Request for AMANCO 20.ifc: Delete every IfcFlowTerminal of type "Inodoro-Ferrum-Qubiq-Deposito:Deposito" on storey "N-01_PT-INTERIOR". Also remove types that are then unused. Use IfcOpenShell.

First a look at what the model holds.

```python
import ifcopenshell
import ifcopenshell.util.element

model = ifcopenshell.open("AMANCO 20.ifc")
print(model.schema)
storey = next(s for s in model.by_type("IfcBuildingStorey") if s.Name == "N-01_PT-INTERIOR")
terminals = [e for e in ifcopenshell.util.element.get_decomposition(storey) if e.is_a("IfcFlowTerminal")]
seen = {}
for e in terminals:
    element_type = ifcopenshell.util.element.get_type(e)
    name = element_type.Name if element_type not in (None, e) else None
    seen[name] = seen.get(name, 0) + 1
for name, count in sorted(seen.items(), key=str):
    print(count, "x", name)
```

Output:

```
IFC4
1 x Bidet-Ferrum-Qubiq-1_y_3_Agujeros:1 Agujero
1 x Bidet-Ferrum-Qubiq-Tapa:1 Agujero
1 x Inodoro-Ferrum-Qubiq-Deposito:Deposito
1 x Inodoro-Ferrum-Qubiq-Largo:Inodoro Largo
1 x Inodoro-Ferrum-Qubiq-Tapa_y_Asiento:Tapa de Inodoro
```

```python
import ifcopenshell
import ifcopenshell.api.root
import ifcopenshell.util.element

model = ifcopenshell.open("AMANCO 20.ifc")

storey = next(s for s in model.by_type("IfcBuildingStorey") if s.Name == "N-01_PT-INTERIOR")
terminals = [e for e in ifcopenshell.util.element.get_decomposition(storey) if e.is_a("IfcFlowTerminal")]
targets = [e for e in terminals if (t := ifcopenshell.util.element.get_type(e)) not in (None, e) and t.Name == "Inodoro-Ferrum-Qubiq-Deposito:Deposito"]
types = {ifcopenshell.util.element.get_type(e) for e in targets} - {None, *targets}

for e in targets:
    ifcopenshell.api.root.remove_product(model, product=e)
print(len(targets), "removed")

unused = [t for t in types if not ifcopenshell.util.element.get_types(t)]
for t in unused:
    ifcopenshell.api.root.remove_product(model, product=t)
print(len(unused), "unused types removed")

model.write("AMANCO 20_edited.ifc")
```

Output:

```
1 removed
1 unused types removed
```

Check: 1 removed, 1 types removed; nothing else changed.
